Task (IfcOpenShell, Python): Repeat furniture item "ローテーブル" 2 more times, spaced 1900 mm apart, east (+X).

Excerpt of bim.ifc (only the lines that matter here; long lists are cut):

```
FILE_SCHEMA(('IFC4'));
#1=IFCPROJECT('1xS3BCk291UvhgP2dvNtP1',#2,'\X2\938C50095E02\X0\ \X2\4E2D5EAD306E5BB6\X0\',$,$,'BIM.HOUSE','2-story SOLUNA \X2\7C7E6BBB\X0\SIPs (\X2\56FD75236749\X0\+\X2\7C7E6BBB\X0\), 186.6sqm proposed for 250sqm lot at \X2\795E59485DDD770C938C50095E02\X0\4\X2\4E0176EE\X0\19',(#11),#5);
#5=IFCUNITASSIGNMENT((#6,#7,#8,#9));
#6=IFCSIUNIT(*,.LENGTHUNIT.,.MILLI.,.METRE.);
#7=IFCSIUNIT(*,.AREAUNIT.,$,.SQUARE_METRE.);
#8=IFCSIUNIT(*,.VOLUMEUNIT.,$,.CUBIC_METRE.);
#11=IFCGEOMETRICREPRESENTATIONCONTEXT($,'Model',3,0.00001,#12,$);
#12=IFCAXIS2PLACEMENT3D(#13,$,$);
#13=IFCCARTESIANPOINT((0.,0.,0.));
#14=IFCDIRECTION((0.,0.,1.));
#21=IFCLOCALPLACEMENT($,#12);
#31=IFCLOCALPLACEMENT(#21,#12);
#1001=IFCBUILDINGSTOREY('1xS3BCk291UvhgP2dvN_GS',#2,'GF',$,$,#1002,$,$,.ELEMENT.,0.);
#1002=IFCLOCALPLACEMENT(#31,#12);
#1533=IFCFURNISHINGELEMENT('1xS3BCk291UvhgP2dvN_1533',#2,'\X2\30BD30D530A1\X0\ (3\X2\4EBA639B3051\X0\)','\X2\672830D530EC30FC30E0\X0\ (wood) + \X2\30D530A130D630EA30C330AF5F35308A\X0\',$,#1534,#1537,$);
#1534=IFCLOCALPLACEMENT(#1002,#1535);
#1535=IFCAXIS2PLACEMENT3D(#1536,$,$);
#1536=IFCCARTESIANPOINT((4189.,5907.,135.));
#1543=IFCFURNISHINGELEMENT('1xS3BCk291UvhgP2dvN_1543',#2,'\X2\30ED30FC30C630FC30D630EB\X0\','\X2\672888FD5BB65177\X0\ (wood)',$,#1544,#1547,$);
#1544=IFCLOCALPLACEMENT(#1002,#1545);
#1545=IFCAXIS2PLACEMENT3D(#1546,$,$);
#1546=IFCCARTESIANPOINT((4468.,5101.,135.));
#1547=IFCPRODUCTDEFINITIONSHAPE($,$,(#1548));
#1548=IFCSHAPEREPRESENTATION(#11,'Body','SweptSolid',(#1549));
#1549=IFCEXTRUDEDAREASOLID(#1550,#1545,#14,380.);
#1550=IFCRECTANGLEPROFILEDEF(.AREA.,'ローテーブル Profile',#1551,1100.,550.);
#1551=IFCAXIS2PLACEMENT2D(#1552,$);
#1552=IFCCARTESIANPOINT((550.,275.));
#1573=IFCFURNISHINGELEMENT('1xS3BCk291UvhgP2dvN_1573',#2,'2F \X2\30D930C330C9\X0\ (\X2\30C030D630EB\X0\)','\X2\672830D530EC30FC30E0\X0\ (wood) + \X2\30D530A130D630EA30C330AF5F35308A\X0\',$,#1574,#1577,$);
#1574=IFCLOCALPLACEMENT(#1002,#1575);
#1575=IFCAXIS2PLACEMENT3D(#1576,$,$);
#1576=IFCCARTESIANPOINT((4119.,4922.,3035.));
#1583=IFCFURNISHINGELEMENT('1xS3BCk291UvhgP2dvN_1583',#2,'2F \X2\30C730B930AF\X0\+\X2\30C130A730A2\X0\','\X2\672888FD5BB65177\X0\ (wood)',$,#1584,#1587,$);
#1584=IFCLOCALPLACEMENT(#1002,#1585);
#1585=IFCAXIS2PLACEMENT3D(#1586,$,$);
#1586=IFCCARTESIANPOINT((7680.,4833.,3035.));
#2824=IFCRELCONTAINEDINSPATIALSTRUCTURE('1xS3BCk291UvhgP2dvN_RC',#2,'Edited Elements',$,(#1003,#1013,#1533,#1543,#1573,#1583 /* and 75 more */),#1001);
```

```python
import numpy as np
import ifcopenshell
import ifcopenshell.api.geometry
import ifcopenshell.api.root
import ifcopenshell.util.element
import ifcopenshell.util.placement
import ifcopenshell.util.unit

model = ifcopenshell.open("bim.ifc")
unit_scale = ifcopenshell.util.unit.calculate_unit_scale(model)


def reuse_history(source, copy):
    """copy_class also copies each property set's owner history, people and application; keep the originals."""
    for rel in copy.IsDefinedBy:
        if rel.is_a("IfcRelDefinesByProperties") and (history := rel.RelatingPropertyDefinition.OwnerHistory):
            rel.RelatingPropertyDefinition.OwnerHistory = source.OwnerHistory
            ifcopenshell.util.element.remove_deep2(model, history)


source = model.by_guid("1xS3BCk291UvhgP2dvN_1543")
base = ifcopenshell.util.placement.get_local_placement(source.ObjectPlacement)
step = np.array([1.0, 0.0, 0.0]) * 1.9 / unit_scale

for i in range(1, 3):
    copy = ifcopenshell.api.root.copy_class(model, product=source)
    copy.Representation = ifcopenshell.util.element.copy_deep(
        model, source.Representation, exclude=["IfcGeometricRepresentationContext", "IfcRepresentationMap"]
    )
    reuse_history(source, copy)
    matrix = base.copy()
    matrix[:3, 3] += i * step
    print("added at", matrix[:3, 3].round(3) + 0.0)
    ifcopenshell.api.geometry.edit_object_placement(model, product=copy, matrix=matrix, is_si=False)

model.write("bim_edited.ifc")
```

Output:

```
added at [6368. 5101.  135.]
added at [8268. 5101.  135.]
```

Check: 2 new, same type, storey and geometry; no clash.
